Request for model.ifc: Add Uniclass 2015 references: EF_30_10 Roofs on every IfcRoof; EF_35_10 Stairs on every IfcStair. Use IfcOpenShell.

First a look at what the model holds.

```python
import ifcopenshell

model = ifcopenshell.open("model.ifc")
print(model.schema)
print("classifications:", [c.Name for c in model.by_type("IfcClassification")])
for ifc_class in ("IfcDoor", "IfcRoof", "IfcStair", "IfcWall", "IfcWindow"):
    print(ifc_class, len(model.by_type(ifc_class)))
```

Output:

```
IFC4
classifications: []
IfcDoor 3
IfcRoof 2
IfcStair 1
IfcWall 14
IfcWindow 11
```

```python
import ifcopenshell
import ifcopenshell.api.classification

model = ifcopenshell.open("model.ifc")

system = ifcopenshell.api.classification.add_classification(model, classification="Uniclass 2015")

codes = {
    "IfcRoof": ("EF_30_10", "Roofs"),
    "IfcStair": ("EF_35_10", "Stairs"),
}
for ifc_class, (code, name) in codes.items():
    products = model.by_type(ifc_class)
    ifcopenshell.api.classification.add_reference(
        model, products=products, classification=system, identification=code, name=name
    )
    print(code, len(products))

model.write("model_v2.ifc")
```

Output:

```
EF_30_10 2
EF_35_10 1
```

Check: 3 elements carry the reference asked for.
